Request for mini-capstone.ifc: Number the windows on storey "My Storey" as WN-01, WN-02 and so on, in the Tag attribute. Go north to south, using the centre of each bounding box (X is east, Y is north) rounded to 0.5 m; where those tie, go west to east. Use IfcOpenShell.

First a look at what the model holds.

```python
import ifcopenshell
import ifcopenshell.util.element
import ifcopenshell.util.placement

model = ifcopenshell.open("mini-capstone.ifc")
print(model.schema)
storey = next(s for s in model.by_type("IfcBuildingStorey") if s.Name == "My Storey")
windows = [e for e in ifcopenshell.util.element.get_decomposition(storey) if e.is_a("IfcWindow")]
for e in sorted(windows, key=lambda e: e.id()):
    origin = ifcopenshell.util.placement.get_local_placement(e.ObjectPlacement)[:3, 3]
    print(e.id(), e.Tag, e.Name, origin.round(2) + 0.0, sep=" | ")
```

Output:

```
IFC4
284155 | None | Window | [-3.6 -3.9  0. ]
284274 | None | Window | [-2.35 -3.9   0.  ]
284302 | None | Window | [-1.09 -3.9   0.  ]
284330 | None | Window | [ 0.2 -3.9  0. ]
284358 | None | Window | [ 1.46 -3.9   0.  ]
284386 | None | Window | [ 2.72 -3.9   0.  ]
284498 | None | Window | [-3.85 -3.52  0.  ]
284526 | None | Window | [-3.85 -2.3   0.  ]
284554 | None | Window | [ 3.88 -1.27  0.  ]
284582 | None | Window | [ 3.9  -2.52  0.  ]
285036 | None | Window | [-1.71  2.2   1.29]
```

```python
import ifcopenshell
import ifcopenshell.geom
import ifcopenshell.util.element
import ifcopenshell.util.shape

model = ifcopenshell.open("mini-capstone.ifc")
settings = ifcopenshell.geom.settings()
settings.set("use-world-coords", True)


def centre(element):
    shape = ifcopenshell.geom.create_shape(settings, element)
    return ifcopenshell.util.shape.get_bbox_centroid(shape.geometry)


storey = next(s for s in model.by_type("IfcBuildingStorey") if s.Name == "My Storey")
windows = [e for e in ifcopenshell.util.element.get_decomposition(storey) if e.is_a("IfcWindow")]

# Insertion points can sit at a corner or the storey origin, so sort by the geometry (in metres).
centres = {e: centre(e) for e in windows}
windows.sort(key=lambda e: (-round(centres[e][1] / 0.5), centres[e][0]))

for i, e in enumerate(windows, start=1):
    number = f"WN-{i:02d}"
    e.Tag = number
    print(e.id(), number)

model.write("mini-capstone_edited.ifc")
```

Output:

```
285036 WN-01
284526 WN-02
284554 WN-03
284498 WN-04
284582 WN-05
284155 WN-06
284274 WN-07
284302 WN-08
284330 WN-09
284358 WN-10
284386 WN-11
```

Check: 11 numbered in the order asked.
